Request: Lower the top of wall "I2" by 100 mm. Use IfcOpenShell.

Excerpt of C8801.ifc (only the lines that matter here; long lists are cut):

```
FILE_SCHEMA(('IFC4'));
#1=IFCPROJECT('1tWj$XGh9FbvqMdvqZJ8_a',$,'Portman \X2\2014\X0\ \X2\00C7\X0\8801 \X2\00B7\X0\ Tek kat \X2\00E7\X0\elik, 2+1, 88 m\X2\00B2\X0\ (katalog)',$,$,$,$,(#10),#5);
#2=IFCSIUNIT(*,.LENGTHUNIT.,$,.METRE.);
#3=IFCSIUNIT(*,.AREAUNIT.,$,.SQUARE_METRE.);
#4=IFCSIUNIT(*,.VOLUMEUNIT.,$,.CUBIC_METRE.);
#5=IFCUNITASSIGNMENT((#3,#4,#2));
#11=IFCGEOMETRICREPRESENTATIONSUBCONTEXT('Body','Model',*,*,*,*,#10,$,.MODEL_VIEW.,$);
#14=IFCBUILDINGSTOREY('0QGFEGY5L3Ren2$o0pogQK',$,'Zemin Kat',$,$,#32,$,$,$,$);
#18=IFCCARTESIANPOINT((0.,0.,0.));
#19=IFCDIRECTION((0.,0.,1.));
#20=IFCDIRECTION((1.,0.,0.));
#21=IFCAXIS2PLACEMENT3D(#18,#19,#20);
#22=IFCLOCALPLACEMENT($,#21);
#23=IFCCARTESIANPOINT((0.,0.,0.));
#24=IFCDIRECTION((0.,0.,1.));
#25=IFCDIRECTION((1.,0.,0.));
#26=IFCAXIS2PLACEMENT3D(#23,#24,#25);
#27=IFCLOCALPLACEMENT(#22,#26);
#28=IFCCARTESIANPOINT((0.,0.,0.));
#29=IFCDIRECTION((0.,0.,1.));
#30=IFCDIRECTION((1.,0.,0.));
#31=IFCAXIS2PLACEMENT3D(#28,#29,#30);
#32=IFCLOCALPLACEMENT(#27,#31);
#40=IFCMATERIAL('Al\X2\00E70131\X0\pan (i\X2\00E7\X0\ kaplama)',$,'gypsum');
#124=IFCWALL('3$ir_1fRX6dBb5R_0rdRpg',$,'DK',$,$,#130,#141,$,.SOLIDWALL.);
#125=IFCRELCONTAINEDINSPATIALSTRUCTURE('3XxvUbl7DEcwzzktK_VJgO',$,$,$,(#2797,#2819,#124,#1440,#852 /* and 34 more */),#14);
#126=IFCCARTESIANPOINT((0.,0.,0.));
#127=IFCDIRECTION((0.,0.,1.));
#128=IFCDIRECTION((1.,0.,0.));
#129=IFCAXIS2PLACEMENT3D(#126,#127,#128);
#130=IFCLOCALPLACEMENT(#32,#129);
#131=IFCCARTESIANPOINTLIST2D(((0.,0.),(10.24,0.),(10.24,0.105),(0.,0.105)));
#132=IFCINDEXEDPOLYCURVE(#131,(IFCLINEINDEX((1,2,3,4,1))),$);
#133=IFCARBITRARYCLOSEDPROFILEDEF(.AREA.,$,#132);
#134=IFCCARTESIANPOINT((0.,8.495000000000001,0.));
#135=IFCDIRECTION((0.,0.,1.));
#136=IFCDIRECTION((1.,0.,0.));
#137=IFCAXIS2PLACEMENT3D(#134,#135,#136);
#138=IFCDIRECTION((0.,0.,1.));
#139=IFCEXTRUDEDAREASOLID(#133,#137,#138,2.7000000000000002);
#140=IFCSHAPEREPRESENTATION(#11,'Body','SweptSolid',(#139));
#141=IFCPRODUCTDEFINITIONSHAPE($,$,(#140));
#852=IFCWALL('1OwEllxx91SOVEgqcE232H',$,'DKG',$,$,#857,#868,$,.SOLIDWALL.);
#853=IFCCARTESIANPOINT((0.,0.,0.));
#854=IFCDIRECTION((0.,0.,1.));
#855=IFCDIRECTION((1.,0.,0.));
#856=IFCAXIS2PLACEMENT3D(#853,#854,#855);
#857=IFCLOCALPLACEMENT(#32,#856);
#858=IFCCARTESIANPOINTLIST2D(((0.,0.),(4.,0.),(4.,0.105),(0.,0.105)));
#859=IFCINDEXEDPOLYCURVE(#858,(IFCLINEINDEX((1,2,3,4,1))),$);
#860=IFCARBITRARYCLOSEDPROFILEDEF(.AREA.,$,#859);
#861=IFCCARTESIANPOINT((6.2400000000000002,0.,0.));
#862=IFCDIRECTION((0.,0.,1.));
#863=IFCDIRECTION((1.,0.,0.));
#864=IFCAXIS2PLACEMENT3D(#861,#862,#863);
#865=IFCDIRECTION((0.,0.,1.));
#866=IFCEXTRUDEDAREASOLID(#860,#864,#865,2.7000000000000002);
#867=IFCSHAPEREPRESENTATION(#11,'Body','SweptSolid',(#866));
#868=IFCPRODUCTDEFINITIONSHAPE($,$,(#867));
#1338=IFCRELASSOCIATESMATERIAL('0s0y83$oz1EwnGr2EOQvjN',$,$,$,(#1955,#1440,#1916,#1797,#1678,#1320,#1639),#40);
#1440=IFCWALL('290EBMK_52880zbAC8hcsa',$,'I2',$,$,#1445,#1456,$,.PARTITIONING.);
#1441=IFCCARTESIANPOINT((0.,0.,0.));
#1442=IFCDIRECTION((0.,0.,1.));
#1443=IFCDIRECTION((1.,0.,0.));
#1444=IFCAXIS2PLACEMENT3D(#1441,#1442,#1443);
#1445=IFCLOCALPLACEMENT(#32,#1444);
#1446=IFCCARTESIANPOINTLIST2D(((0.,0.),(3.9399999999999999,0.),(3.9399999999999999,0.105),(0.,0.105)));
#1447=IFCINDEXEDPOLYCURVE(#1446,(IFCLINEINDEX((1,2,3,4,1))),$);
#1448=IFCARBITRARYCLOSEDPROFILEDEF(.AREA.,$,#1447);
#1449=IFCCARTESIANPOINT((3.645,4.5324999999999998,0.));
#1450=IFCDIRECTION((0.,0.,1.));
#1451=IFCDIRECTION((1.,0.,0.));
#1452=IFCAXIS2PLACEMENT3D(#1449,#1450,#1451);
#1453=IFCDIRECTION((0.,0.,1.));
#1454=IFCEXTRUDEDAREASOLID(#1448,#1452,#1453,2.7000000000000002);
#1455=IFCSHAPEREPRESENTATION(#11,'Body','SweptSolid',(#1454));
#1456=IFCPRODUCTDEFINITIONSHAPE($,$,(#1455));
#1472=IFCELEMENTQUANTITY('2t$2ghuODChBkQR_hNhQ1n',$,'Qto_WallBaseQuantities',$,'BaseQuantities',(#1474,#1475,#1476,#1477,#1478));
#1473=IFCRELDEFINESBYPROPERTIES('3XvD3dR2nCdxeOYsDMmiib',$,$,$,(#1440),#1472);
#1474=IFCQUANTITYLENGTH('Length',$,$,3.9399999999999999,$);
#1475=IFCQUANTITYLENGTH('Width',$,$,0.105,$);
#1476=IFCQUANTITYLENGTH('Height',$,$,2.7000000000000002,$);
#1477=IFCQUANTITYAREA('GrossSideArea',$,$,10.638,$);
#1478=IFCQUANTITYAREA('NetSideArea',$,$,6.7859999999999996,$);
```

```python
import ifcopenshell
import ifcopenshell.api.pset
import ifcopenshell.geom
import ifcopenshell.util.element
import ifcopenshell.util.representation
import ifcopenshell.util.shape
import ifcopenshell.util.unit

model = ifcopenshell.open("C8801.ifc")
unit_scale = ifcopenshell.util.unit.calculate_unit_scale(model)
area_scale = ifcopenshell.util.unit.calculate_unit_scale(model, "AREAUNIT")
settings = ifcopenshell.geom.settings()


def volume(element):
    """Net volume in cubic metres, openings subtracted."""
    shape = ifcopenshell.geom.create_shape(settings, element)
    return ifcopenshell.util.shape.get_volume(shape.geometry)


wall = model.by_id(1440)
before = volume(wall)

body = ifcopenshell.util.representation.get_representation(wall, "Model", "Body")
solid = body.Items[0]
old_height = solid.Depth
solid.Depth -= 0.1 / unit_scale
after = volume(wall)
thickness = 0.105  # wall thickness in metres

# Update the stored height, areas and volumes.
qto = model.by_id(ifcopenshell.util.element.get_pset(wall, "Qto_WallBaseQuantities", should_inherit=False)["id"])
ifcopenshell.api.pset.edit_qto(model, qto=qto, properties={
    "Height": solid.Depth,
    "GrossSideArea": ifcopenshell.util.element.get_pset(wall, "Qto_WallBaseQuantities", "GrossSideArea") * solid.Depth / old_height,
    "NetSideArea": after / thickness / area_scale,
})

print(f"height {old_height:g} -> {solid.Depth:g}, volume {before:.3f} -> {after:.3f} m3")

model.write("C8801_rev.ifc")
```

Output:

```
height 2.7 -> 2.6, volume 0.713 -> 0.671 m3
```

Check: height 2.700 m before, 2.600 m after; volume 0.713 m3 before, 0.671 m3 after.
